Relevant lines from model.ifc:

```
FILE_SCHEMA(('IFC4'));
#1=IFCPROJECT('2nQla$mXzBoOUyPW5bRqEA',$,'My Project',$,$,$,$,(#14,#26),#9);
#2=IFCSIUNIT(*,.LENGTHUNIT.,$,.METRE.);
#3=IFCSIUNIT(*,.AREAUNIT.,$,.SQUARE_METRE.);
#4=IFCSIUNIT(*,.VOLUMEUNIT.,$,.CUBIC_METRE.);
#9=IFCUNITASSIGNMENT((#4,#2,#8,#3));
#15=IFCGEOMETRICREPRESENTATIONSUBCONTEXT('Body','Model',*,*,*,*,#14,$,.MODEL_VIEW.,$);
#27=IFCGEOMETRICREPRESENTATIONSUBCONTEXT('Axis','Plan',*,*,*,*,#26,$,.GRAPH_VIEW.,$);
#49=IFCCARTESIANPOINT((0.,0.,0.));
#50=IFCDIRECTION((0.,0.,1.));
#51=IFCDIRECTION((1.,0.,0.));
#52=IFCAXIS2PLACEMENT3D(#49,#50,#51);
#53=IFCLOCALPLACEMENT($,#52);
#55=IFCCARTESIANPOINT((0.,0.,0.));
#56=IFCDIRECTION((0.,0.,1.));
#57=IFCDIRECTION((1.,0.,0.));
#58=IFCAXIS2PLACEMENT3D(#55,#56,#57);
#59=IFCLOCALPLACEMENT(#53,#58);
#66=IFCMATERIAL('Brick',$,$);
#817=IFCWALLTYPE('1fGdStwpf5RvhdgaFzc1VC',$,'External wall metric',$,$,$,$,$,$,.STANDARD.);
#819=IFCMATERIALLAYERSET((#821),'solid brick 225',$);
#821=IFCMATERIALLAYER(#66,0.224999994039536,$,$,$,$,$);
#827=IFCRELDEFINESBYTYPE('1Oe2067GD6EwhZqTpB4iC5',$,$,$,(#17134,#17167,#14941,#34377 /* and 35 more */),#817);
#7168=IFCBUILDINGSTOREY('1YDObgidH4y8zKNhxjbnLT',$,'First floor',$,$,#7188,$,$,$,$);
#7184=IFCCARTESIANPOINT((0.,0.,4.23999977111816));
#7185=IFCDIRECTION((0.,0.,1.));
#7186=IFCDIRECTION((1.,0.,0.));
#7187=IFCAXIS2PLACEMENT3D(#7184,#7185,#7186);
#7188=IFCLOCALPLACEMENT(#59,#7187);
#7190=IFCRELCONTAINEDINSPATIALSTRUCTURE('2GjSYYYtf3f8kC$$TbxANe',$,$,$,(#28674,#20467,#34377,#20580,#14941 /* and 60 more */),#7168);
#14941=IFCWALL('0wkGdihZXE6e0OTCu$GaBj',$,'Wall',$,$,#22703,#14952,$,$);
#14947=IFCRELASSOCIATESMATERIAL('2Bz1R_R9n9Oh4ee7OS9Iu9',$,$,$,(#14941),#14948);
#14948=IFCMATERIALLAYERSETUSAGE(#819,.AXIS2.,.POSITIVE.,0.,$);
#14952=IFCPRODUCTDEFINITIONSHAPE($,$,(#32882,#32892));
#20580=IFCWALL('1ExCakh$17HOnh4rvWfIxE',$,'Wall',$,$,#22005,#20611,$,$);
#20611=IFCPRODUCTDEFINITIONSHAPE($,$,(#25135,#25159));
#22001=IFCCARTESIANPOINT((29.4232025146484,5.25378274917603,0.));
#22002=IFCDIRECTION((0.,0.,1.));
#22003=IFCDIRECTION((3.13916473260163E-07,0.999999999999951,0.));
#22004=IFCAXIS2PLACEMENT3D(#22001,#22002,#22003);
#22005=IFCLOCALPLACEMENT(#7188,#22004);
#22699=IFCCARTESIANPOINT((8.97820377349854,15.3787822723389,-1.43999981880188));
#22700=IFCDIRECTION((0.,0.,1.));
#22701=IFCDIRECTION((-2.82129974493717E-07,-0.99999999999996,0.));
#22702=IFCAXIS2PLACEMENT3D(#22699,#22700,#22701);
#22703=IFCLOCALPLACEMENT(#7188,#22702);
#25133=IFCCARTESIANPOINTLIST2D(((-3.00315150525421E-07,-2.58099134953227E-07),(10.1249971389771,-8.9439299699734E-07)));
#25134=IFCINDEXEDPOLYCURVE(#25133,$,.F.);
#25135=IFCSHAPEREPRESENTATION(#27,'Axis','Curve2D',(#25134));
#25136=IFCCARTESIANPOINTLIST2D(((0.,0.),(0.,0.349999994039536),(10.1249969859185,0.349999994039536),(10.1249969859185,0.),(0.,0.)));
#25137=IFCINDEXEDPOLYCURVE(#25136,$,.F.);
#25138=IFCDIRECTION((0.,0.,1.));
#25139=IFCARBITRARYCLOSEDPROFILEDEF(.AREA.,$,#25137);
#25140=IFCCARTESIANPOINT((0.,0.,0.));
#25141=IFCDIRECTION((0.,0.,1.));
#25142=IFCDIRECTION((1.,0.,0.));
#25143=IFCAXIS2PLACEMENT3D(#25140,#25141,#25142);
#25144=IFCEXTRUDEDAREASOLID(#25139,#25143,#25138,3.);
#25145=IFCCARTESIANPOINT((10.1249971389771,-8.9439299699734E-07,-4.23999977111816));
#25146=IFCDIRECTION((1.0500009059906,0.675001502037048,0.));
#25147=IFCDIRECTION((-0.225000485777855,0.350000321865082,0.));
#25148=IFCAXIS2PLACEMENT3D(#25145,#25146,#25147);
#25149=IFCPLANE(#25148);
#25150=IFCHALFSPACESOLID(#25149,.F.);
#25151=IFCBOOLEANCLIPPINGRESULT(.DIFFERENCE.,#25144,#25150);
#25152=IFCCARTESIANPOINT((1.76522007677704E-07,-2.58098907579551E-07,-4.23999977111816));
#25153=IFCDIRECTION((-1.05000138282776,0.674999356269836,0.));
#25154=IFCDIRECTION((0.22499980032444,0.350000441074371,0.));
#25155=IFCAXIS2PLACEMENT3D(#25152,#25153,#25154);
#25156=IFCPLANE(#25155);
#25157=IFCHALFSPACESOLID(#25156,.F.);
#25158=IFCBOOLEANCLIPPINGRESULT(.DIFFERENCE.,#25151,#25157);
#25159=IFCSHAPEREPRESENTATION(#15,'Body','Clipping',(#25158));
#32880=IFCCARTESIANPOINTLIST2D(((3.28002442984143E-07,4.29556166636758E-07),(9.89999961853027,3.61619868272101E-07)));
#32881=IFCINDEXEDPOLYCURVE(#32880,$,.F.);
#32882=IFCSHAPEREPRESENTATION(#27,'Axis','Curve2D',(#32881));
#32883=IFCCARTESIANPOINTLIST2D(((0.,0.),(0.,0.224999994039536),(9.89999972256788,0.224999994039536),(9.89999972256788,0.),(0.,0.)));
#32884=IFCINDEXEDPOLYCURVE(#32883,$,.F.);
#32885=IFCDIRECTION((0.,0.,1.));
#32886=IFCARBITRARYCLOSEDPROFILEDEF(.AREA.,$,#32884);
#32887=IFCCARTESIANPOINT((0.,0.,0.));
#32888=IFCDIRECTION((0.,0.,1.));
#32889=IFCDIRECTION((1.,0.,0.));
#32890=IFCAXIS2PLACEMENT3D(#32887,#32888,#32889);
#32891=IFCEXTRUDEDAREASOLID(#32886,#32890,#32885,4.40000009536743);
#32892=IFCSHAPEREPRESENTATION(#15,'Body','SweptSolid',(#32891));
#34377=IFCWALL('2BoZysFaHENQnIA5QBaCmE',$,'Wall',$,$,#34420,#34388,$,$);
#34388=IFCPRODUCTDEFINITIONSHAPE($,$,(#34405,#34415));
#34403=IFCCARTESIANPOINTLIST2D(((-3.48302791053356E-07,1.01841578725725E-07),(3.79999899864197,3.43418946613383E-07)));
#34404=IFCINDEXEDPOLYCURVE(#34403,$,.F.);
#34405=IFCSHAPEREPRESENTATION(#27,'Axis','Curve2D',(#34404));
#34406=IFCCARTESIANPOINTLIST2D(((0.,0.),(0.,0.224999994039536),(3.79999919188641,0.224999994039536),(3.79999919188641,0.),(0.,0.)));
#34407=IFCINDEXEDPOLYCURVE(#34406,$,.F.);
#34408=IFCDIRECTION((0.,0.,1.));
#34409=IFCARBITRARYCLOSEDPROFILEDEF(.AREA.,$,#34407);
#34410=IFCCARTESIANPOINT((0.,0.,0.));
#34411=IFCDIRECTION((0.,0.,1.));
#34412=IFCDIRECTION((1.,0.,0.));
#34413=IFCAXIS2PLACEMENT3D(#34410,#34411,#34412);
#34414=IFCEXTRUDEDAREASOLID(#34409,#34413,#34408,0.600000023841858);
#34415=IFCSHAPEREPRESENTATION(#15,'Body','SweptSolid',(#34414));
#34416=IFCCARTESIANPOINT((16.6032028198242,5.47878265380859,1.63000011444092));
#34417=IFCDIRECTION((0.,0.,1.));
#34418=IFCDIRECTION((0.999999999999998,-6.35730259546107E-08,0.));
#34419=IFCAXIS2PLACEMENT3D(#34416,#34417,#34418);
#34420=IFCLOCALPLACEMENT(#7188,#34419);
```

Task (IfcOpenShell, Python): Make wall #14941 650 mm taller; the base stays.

```python
import ifcopenshell
import ifcopenshell.geom
import ifcopenshell.util.representation
import ifcopenshell.util.shape
import ifcopenshell.util.unit

model = ifcopenshell.open("model.ifc")
unit_scale = ifcopenshell.util.unit.calculate_unit_scale(model)
settings = ifcopenshell.geom.settings()


def volume(element):
    """Net volume in cubic metres, openings subtracted."""
    shape = ifcopenshell.geom.create_shape(settings, element)
    return ifcopenshell.util.shape.get_volume(shape.geometry)


wall = model.by_id(14941)
before = volume(wall)

body = ifcopenshell.util.representation.get_representation(wall, "Model", "Body")
solid = body.Items[0]
old_height = solid.Depth
solid.Depth += 0.65 / unit_scale
after = volume(wall)

print(f"height {old_height:g} -> {solid.Depth:g}, volume {before:.3f} -> {after:.3f} m3")

model.write("model-out.ifc")
```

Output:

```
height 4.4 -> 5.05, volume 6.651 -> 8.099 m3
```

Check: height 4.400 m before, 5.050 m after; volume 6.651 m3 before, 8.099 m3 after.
